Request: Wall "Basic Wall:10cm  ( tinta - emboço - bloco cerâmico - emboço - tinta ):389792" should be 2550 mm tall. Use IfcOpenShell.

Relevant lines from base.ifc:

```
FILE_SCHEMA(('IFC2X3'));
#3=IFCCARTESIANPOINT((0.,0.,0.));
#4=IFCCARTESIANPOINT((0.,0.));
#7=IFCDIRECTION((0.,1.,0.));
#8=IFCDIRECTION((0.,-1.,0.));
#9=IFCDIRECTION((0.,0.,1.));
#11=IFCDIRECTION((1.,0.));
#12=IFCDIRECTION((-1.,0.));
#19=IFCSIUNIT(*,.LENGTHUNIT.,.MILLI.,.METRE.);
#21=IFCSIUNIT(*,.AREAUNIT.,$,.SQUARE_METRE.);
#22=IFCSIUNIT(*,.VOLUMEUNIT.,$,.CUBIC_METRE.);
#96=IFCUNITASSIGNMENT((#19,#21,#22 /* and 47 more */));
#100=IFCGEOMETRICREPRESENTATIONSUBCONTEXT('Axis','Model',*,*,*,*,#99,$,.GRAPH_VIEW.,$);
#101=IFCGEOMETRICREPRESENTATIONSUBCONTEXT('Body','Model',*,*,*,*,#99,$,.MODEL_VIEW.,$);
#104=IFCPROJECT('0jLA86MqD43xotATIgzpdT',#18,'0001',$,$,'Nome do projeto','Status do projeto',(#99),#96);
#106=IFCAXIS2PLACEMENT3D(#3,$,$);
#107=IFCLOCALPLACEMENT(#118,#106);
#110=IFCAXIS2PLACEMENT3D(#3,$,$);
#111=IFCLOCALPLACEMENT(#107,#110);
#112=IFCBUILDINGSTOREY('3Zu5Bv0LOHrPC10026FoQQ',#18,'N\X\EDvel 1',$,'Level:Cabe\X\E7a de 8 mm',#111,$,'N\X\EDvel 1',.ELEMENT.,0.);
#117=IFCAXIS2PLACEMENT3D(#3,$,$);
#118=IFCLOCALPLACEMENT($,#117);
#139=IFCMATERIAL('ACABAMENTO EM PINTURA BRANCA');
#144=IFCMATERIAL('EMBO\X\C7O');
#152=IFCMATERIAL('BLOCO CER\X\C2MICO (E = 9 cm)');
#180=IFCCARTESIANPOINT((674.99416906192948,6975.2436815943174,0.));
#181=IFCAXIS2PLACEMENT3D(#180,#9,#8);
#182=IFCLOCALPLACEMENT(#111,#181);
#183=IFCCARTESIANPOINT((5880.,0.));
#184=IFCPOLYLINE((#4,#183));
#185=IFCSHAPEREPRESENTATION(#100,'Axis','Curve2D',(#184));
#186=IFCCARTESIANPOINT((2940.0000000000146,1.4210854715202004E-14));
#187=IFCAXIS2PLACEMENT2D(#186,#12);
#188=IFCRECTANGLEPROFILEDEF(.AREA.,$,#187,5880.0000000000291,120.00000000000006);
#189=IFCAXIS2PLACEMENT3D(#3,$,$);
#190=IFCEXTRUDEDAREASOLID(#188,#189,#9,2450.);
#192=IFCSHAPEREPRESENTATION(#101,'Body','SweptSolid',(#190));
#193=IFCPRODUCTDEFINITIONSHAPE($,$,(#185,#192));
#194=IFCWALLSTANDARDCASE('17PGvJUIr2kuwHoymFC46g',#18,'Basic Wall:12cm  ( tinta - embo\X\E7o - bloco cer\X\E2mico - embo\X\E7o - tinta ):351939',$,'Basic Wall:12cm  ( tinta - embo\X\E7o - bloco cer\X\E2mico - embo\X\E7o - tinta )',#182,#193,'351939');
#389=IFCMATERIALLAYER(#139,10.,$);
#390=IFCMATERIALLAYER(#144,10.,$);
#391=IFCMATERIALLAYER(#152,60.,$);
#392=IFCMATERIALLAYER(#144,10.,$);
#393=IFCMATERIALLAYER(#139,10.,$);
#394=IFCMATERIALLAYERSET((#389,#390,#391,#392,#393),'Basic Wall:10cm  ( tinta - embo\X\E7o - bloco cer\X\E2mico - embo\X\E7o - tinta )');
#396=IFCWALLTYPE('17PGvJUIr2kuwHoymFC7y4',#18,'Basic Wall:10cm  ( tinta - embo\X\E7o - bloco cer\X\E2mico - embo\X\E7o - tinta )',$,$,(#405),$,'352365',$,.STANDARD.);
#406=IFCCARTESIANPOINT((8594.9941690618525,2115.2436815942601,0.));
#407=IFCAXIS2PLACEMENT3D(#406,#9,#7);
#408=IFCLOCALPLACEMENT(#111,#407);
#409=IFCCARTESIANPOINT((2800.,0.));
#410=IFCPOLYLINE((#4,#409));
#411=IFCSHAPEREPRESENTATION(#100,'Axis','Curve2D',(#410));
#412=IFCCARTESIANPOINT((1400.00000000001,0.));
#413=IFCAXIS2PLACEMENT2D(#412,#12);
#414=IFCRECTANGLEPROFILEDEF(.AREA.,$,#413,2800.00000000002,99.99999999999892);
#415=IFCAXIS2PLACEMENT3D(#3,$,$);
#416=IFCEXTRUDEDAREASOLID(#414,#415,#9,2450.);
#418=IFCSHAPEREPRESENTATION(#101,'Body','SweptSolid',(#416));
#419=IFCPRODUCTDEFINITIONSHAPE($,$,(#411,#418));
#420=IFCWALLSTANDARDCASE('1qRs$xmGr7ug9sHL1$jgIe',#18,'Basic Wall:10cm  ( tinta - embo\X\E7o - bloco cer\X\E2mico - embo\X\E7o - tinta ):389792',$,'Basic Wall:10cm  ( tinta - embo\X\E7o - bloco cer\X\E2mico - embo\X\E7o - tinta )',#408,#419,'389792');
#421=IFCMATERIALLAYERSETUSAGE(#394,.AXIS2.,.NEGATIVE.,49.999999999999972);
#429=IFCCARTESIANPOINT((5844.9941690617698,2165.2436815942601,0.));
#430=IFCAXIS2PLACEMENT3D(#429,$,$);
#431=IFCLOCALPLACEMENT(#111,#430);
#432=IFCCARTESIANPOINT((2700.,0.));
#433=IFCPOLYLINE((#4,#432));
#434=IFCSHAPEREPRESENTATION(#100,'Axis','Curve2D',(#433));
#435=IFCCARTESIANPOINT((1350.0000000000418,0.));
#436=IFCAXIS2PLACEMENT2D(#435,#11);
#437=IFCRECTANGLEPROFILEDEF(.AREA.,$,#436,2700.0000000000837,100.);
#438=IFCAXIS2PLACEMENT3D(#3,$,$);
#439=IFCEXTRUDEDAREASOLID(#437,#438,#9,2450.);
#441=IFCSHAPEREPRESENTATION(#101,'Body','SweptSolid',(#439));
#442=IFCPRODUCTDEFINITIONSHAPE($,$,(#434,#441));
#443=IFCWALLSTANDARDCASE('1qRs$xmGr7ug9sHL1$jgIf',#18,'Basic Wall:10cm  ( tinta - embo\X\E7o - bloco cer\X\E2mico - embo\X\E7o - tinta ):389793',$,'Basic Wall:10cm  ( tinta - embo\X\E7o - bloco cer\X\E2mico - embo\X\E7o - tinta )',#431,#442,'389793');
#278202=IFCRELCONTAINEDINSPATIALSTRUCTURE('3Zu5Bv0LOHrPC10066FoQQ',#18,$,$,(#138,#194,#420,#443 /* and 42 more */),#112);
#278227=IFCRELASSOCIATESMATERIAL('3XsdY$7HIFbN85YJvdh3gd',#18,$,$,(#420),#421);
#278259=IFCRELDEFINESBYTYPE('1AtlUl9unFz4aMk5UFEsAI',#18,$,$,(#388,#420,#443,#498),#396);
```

```python
import ifcopenshell
import ifcopenshell.geom
import ifcopenshell.util.representation
import ifcopenshell.util.shape

model = ifcopenshell.open("base.ifc")
settings = ifcopenshell.geom.settings()


def volume(element):
    """Net volume in cubic metres, openings subtracted."""
    shape = ifcopenshell.geom.create_shape(settings, element)
    return ifcopenshell.util.shape.get_volume(shape.geometry)


wall = model.by_guid("1qRs$xmGr7ug9sHL1$jgIe")
before = volume(wall)

body = ifcopenshell.util.representation.get_representation(wall, "Model", "Body")
solid = body.Items[0]
old_height = solid.Depth
solid.Depth = 2550.0
after = volume(wall)

print(f"height {old_height:g} -> {solid.Depth:g}, volume {before:.3f} -> {after:.3f} m3")

model.write("base_v2.ifc")
```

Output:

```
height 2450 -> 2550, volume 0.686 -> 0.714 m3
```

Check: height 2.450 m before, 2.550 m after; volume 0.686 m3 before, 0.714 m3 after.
